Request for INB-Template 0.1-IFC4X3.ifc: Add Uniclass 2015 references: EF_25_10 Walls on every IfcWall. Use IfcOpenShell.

First a look at what the model holds.

```python
import ifcopenshell

model = ifcopenshell.open("INB-Template 0.1-IFC4X3.ifc")
print(model.schema)
print("classifications:", [c.Name for c in model.by_type("IfcClassification")])
for ifc_class in ("IfcDoor", "IfcRoof", "IfcStair", "IfcWall", "IfcWindow"):
    print(ifc_class, len(model.by_type(ifc_class)))
```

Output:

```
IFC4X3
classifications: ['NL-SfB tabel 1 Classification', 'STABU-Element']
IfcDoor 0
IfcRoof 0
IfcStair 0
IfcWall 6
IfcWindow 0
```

```python
import ifcopenshell
import ifcopenshell.api.classification

model = ifcopenshell.open("INB-Template 0.1-IFC4X3.ifc")

system = ifcopenshell.api.classification.add_classification(model, classification="Uniclass 2015")

codes = {
    "IfcWall": ("EF_25_10", "Walls"),
}
for ifc_class, (code, name) in codes.items():
    products = model.by_type(ifc_class)
    ifcopenshell.api.classification.add_reference(
        model, products=products, classification=system, identification=code, name=name
    )
    print(code, len(products))

model.write("INB-Template 0.1-IFC4X3_v2.ifc")
```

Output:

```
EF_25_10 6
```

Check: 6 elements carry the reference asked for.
